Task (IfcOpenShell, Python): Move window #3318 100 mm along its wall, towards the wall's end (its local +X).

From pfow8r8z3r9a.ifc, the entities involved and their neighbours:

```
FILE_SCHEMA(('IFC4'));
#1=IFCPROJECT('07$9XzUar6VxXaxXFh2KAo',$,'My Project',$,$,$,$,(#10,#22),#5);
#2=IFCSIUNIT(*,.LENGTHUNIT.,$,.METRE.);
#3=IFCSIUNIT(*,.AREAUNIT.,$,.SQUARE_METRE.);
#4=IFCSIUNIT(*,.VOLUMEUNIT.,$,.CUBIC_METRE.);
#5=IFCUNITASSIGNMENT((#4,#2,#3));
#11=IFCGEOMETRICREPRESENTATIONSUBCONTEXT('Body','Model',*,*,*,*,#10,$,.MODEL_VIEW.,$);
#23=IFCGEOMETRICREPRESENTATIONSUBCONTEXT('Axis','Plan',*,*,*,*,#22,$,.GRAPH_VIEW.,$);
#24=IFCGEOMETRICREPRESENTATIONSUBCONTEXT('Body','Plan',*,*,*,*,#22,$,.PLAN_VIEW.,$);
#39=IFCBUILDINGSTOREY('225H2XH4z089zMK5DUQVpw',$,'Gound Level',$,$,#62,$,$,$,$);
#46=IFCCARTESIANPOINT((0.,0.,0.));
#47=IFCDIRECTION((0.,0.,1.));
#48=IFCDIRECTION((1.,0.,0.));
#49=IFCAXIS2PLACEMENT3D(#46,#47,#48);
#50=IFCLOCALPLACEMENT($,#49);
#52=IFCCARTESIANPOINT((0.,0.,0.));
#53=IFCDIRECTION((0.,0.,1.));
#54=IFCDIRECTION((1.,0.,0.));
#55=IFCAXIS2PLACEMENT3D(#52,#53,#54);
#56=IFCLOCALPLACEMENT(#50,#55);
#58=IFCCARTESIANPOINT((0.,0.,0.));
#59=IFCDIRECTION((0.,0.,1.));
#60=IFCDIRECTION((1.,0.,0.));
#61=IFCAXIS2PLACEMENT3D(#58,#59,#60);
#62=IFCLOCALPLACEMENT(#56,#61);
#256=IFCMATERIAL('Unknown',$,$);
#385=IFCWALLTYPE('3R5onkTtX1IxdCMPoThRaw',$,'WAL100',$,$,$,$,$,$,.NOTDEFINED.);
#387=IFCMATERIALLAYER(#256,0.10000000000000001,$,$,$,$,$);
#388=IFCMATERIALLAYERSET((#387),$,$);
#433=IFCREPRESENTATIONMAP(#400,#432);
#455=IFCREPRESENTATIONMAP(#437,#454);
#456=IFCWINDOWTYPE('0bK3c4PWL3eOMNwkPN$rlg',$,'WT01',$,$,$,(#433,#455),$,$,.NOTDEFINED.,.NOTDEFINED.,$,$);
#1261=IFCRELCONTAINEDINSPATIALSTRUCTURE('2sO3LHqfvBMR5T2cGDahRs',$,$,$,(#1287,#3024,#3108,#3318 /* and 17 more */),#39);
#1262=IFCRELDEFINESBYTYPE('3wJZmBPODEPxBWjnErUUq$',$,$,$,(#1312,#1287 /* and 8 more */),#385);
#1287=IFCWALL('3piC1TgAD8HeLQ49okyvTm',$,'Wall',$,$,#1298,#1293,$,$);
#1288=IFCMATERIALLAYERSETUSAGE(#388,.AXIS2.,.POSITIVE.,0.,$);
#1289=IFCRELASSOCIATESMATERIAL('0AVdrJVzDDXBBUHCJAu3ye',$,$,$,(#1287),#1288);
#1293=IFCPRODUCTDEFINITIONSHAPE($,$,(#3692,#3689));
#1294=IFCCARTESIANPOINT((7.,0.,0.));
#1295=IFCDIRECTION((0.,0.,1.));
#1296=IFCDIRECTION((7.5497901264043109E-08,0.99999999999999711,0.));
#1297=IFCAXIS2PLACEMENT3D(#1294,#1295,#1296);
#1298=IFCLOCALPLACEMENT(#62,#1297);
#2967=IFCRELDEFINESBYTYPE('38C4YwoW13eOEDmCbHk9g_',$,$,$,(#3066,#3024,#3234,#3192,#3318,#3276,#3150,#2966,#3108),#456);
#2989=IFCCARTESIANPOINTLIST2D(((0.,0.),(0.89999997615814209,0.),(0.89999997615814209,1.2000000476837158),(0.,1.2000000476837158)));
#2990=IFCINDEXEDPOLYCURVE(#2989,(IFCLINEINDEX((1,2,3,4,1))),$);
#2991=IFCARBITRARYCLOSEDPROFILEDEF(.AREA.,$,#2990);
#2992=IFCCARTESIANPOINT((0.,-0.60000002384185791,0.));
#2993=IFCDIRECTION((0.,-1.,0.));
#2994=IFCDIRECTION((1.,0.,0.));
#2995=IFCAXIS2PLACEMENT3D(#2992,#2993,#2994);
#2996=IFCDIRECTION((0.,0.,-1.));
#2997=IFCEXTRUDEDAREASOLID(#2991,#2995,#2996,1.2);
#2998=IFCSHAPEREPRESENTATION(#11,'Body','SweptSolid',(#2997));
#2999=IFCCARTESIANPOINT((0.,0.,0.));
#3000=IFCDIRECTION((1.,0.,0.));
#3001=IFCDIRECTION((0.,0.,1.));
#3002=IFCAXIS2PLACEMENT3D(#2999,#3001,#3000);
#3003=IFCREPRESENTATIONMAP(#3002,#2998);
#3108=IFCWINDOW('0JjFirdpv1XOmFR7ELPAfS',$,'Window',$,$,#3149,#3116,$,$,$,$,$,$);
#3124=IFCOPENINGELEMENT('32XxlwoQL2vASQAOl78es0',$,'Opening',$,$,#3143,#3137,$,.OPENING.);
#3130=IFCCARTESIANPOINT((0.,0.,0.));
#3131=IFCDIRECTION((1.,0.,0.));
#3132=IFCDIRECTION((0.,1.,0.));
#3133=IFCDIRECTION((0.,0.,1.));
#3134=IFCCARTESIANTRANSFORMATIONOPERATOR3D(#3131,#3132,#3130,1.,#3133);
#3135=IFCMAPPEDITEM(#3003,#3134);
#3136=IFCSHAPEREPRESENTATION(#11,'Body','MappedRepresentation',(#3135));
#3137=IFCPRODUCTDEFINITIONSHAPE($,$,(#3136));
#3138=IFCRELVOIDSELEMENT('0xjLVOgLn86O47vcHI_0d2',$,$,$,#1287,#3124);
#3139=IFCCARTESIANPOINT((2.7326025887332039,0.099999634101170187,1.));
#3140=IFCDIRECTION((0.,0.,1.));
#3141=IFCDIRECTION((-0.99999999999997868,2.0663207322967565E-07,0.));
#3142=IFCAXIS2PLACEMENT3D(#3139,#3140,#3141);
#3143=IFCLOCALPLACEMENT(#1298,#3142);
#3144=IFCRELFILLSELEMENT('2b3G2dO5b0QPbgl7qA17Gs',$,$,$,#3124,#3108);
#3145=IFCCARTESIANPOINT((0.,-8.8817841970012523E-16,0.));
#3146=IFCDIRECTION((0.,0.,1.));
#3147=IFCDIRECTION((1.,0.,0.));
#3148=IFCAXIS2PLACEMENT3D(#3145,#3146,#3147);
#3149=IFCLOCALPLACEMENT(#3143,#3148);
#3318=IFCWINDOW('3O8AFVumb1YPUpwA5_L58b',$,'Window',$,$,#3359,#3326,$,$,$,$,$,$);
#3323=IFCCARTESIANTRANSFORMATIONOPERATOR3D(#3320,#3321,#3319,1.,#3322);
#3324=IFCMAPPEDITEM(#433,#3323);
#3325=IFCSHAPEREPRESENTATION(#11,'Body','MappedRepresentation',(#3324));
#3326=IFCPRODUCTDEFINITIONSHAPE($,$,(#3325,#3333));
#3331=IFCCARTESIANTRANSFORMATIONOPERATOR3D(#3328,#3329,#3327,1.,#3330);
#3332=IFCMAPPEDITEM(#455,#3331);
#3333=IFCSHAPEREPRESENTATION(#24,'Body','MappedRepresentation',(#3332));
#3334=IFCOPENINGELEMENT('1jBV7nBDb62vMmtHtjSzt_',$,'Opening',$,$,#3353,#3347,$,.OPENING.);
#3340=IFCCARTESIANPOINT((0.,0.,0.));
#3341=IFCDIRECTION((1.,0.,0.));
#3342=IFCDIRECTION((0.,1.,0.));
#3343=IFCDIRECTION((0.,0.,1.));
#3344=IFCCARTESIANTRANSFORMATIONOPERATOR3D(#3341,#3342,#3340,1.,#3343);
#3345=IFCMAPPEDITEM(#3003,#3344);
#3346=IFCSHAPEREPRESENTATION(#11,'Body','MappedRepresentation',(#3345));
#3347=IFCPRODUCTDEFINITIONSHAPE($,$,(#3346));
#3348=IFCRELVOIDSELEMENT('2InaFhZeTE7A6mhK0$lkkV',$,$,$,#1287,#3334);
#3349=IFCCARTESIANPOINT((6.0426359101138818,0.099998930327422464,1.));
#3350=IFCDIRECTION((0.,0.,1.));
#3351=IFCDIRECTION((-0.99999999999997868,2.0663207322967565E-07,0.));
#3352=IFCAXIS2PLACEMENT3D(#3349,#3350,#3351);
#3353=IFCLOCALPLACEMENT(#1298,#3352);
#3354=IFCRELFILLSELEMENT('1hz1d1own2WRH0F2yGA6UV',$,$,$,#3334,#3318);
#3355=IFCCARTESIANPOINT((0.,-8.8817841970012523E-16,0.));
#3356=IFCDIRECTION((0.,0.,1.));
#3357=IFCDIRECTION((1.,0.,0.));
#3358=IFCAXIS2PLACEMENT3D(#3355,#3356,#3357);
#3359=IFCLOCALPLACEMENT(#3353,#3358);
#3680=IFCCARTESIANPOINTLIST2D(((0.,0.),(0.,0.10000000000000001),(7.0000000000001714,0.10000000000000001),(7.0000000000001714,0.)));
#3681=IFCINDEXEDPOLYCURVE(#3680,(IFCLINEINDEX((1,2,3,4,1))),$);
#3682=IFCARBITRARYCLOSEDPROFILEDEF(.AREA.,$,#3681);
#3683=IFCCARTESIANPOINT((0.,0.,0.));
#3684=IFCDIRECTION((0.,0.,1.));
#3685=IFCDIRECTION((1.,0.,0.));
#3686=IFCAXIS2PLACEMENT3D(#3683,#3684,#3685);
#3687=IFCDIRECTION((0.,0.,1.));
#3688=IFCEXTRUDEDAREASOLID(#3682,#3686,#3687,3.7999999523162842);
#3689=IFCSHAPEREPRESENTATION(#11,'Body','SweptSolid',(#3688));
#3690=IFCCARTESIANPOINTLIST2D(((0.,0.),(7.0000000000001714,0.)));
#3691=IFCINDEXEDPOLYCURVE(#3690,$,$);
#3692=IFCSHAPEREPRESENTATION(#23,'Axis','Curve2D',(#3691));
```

```python
import ifcopenshell
import ifcopenshell.api.geometry
import ifcopenshell.util.placement

model = ifcopenshell.open("pfow8r8z3r9a.ifc")

window = model.by_guid("3O8AFVumb1YPUpwA5_L58b")
opening = window.FillsVoids[0].RelatingOpeningElement
wall = opening.VoidsElements[0].RelatingBuildingElement

wall_matrix = ifcopenshell.util.placement.get_local_placement(wall.ObjectPlacement)
shift = wall_matrix[:3, 0] * 0.1
before = ifcopenshell.util.placement.get_local_placement(window.ObjectPlacement)[:3, 3].copy()

# The window is placed relative to its opening, so it follows when the opening moves.
matrix = ifcopenshell.util.placement.get_local_placement(opening.ObjectPlacement)
matrix[:3, 3] += shift
ifcopenshell.api.geometry.edit_object_placement(
    model, product=opening, matrix=matrix, is_si=False, should_transform_children=True
)

after = ifcopenshell.util.placement.get_local_placement(window.ObjectPlacement)[:3, 3]
print("window moved by", (after - before).round(3) + 0.0)

model.write("pfow8r8z3r9a-out.ifc")
```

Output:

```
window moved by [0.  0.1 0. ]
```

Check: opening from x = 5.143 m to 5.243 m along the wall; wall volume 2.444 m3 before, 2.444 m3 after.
